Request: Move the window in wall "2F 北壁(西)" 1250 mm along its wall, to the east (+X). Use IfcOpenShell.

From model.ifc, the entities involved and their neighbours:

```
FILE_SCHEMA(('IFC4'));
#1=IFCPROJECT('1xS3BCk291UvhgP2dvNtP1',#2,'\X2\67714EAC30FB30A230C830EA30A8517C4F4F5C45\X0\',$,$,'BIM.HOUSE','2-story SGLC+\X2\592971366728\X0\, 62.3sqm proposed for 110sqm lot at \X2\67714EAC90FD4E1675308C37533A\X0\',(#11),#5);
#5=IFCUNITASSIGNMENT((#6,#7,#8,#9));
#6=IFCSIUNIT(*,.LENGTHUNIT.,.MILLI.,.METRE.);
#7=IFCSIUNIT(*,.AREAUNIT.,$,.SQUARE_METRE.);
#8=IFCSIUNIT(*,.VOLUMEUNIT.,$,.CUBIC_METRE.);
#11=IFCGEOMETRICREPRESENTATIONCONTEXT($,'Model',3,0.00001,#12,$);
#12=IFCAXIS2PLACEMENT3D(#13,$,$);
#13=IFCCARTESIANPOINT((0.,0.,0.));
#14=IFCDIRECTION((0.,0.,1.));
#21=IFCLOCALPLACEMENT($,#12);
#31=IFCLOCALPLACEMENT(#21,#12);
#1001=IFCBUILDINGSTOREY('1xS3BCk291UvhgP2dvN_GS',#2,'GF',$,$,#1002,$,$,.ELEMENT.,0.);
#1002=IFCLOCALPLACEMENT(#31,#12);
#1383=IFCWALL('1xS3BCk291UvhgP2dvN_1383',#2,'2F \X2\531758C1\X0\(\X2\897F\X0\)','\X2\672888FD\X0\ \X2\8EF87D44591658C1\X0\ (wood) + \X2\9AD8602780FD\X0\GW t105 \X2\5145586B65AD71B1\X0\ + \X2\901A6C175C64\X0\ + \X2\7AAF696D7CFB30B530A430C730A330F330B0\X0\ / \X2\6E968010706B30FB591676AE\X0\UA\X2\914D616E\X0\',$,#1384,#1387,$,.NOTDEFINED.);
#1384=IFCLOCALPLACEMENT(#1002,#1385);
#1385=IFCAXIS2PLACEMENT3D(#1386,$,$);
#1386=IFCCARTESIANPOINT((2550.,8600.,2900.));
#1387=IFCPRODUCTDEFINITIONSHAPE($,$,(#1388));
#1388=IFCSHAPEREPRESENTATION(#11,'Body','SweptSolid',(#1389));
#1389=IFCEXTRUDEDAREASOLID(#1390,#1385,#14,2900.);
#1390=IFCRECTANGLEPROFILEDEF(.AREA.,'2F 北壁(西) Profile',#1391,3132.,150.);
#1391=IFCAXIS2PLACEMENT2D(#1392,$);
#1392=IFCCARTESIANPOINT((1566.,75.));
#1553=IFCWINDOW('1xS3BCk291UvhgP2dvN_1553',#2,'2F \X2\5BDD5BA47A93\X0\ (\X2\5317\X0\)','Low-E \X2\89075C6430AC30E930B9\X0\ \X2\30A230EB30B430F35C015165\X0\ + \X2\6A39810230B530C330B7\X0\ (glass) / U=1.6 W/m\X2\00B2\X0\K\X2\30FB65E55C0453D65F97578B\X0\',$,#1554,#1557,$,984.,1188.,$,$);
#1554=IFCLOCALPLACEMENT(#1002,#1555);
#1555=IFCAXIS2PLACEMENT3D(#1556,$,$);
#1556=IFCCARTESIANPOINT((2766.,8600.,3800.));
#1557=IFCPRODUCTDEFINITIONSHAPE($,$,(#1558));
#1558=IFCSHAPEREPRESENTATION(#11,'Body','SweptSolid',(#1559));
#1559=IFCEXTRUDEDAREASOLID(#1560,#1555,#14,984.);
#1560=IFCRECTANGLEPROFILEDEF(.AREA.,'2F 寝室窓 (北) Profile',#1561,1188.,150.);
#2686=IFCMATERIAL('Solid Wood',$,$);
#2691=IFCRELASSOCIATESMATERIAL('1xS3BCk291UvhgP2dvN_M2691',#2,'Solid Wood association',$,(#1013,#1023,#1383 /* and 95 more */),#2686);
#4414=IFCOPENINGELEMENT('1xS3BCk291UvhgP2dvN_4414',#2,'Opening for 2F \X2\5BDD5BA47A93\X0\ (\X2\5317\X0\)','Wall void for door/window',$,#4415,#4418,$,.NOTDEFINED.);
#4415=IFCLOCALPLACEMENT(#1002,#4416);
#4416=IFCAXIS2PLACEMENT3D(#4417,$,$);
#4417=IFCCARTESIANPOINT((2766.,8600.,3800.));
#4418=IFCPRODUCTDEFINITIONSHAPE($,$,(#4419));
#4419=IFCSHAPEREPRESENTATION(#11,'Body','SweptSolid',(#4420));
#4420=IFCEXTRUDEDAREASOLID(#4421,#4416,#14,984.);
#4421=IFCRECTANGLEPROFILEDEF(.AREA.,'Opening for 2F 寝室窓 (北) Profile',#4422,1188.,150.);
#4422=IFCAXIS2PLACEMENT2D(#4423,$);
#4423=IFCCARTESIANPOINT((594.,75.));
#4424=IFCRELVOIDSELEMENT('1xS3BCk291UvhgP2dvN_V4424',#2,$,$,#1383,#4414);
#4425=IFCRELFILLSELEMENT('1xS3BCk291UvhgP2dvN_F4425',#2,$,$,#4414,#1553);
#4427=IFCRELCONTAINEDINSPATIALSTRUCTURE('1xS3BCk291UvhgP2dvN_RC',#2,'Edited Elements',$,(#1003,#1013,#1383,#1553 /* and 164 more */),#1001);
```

```python
import ifcopenshell
import ifcopenshell.api.geometry
import ifcopenshell.util.placement

model = ifcopenshell.open("model.ifc")

window = model.by_guid("1xS3BCk291UvhgP2dvN_1553")
opening = window.FillsVoids[0].RelatingOpeningElement
wall = opening.VoidsElements[0].RelatingBuildingElement

wall_matrix = ifcopenshell.util.placement.get_local_placement(wall.ObjectPlacement)
shift = wall_matrix[:3, 0] * 1250.0
before = ifcopenshell.util.placement.get_local_placement(window.ObjectPlacement)[:3, 3].copy()

# The window is not placed relative to its opening, so move both.
for product in (opening, window):
    matrix = ifcopenshell.util.placement.get_local_placement(product.ObjectPlacement)
    matrix[:3, 3] += shift
    ifcopenshell.api.geometry.edit_object_placement(model, product=product, matrix=matrix, is_si=False)

after = ifcopenshell.util.placement.get_local_placement(window.ObjectPlacement)[:3, 3]
print("window moved by", (after - before).round(3) + 0.0)

model.write("model_rev.ifc")
```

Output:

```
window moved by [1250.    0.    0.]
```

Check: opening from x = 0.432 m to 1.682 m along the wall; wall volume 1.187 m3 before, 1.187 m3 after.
